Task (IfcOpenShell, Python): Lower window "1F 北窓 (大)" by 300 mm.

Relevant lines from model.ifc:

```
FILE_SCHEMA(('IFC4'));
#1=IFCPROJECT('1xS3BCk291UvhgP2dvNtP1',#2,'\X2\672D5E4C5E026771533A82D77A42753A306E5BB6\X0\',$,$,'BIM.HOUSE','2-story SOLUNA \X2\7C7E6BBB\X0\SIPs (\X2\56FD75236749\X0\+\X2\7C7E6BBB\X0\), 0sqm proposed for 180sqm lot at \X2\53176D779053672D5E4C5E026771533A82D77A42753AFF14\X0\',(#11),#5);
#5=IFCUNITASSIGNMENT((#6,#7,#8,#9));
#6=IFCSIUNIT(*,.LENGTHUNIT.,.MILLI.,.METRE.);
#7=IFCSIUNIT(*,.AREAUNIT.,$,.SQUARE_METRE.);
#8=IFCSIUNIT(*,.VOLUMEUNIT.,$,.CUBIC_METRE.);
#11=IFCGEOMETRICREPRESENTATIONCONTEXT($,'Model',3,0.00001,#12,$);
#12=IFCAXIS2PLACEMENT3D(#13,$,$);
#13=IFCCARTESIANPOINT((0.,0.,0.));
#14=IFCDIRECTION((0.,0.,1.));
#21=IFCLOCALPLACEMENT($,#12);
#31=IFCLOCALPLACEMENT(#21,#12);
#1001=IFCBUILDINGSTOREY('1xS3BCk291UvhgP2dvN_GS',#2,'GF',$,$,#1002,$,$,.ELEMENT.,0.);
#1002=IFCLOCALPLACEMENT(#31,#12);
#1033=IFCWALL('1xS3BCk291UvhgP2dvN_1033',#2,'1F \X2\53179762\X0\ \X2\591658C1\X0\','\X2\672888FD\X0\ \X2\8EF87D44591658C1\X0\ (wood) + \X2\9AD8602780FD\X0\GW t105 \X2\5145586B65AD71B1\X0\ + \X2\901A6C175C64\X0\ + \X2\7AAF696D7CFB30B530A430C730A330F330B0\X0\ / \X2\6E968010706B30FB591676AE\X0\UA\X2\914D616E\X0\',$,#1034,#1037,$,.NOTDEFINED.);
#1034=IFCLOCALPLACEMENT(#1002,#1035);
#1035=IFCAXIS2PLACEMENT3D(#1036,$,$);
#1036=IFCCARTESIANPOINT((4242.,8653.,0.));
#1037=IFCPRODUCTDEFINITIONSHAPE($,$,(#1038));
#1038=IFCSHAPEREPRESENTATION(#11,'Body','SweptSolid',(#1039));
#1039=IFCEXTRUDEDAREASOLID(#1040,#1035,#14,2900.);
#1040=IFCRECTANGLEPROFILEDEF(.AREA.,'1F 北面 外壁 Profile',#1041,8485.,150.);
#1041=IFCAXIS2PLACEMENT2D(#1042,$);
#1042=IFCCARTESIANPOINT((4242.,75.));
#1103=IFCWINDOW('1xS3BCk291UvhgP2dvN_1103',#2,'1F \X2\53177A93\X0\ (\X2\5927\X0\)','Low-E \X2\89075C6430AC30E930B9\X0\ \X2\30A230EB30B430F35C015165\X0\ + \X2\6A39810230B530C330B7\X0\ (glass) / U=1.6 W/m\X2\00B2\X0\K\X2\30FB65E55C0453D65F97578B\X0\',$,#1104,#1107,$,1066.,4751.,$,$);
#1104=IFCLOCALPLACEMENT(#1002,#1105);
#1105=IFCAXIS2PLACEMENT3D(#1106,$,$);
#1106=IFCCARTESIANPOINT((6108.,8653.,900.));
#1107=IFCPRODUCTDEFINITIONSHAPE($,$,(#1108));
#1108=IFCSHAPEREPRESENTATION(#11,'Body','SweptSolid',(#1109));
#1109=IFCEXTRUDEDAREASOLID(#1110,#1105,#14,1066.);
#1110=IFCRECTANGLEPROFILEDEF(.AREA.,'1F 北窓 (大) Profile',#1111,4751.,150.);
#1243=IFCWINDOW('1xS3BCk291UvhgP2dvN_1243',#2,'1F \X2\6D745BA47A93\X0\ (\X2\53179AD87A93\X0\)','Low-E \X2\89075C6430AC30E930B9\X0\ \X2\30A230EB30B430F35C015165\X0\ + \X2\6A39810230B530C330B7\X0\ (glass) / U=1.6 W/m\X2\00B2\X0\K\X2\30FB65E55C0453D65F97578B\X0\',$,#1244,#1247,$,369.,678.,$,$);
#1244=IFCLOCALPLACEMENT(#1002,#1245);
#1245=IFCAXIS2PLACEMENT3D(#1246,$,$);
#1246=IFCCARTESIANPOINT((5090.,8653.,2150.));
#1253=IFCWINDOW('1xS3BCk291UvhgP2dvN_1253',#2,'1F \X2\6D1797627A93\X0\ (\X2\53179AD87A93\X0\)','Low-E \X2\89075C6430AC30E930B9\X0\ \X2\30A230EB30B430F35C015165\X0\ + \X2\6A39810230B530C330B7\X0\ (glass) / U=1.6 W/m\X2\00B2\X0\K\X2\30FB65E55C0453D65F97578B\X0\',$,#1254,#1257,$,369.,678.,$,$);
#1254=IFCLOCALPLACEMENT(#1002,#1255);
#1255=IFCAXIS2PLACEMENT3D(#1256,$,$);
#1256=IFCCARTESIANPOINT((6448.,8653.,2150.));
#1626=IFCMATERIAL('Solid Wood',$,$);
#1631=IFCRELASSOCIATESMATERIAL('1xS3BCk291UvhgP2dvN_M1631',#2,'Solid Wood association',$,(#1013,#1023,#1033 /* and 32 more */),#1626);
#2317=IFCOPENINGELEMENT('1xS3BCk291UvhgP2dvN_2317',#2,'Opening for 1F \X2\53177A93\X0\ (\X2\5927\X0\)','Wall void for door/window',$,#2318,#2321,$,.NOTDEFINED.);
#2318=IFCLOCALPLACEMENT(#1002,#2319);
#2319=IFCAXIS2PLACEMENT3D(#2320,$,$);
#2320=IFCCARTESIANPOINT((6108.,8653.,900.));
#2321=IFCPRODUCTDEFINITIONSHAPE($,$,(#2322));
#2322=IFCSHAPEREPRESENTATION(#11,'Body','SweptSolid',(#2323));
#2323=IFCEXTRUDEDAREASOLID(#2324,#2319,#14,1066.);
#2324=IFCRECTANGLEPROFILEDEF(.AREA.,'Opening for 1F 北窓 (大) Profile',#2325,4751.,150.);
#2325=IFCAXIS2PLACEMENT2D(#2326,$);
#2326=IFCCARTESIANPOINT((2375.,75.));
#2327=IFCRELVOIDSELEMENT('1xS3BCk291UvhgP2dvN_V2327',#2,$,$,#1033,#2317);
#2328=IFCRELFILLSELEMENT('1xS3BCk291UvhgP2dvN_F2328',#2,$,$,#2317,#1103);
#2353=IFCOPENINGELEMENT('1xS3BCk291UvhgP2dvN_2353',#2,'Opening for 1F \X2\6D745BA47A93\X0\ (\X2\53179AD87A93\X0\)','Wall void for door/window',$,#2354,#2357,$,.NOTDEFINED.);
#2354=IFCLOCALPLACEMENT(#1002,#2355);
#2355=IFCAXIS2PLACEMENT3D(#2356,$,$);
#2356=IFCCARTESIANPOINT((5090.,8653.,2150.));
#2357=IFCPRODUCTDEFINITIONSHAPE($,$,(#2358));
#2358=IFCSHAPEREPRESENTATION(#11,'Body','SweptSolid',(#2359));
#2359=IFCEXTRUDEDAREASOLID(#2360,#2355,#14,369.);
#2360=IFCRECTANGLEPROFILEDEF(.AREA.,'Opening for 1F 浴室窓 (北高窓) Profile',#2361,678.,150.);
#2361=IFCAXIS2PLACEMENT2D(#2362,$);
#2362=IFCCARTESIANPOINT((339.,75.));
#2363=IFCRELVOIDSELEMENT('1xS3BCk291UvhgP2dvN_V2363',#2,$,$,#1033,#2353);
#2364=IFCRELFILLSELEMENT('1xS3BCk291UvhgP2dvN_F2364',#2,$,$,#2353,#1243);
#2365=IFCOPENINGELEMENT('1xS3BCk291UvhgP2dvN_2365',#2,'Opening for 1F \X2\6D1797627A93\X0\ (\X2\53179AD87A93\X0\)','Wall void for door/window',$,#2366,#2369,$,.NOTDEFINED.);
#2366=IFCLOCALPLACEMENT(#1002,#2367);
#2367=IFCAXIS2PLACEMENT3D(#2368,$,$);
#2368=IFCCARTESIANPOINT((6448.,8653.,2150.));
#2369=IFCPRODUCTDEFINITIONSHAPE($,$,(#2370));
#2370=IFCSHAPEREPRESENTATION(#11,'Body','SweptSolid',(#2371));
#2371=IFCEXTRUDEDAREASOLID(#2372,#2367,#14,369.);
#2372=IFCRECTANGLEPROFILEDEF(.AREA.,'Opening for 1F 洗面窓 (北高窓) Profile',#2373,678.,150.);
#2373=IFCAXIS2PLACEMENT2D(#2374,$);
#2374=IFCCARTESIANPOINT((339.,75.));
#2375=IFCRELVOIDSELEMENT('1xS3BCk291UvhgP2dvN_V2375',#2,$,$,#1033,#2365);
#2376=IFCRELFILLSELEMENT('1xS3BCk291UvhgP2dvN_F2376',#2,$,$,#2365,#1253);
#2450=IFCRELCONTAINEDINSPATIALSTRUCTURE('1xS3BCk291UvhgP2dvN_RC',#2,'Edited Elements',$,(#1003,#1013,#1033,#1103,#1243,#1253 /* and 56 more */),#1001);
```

```python
import numpy as np
import ifcopenshell
import ifcopenshell.api.geometry
import ifcopenshell.util.placement
import ifcopenshell.util.unit

model = ifcopenshell.open("model.ifc")
unit_scale = ifcopenshell.util.unit.calculate_unit_scale(model)

window = model.by_guid("1xS3BCk291UvhgP2dvN_1103")
opening = window.FillsVoids[0].RelatingOpeningElement
dz = -300.0

shift = np.array([0.0, 0.0, dz])
# The window is not placed relative to its opening, so move both.
for product in (opening, window):
    matrix = ifcopenshell.util.placement.get_local_placement(product.ObjectPlacement)
    matrix[:3, 3] += shift
    ifcopenshell.api.geometry.edit_object_placement(model, product=product, matrix=matrix, is_si=False)

print(f"moved by {dz * unit_scale:+.3f} m")

model.write("model-out.ifc")
```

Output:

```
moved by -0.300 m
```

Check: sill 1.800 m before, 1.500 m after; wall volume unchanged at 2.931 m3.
